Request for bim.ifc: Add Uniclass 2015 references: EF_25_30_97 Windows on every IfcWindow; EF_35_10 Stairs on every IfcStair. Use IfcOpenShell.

First a look at what the model holds.

```python
import ifcopenshell

model = ifcopenshell.open("bim.ifc")
print(model.schema)
print("classifications:", [c.Name for c in model.by_type("IfcClassification")])
for ifc_class in ("IfcDoor", "IfcRoof", "IfcStair", "IfcWall", "IfcWindow"):
    print(ifc_class, len(model.by_type(ifc_class)))
```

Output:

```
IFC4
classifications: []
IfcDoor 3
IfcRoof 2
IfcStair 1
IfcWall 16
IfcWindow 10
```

```python
import ifcopenshell
import ifcopenshell.api.classification

model = ifcopenshell.open("bim.ifc")

system = ifcopenshell.api.classification.add_classification(model, classification="Uniclass 2015")

codes = {
    "IfcWindow": ("EF_25_30_97", "Windows"),
    "IfcStair": ("EF_35_10", "Stairs"),
}
for ifc_class, (code, name) in codes.items():
    products = model.by_type(ifc_class)
    ifcopenshell.api.classification.add_reference(
        model, products=products, classification=system, identification=code, name=name
    )
    print(code, len(products))

model.write("bim-out.ifc")
```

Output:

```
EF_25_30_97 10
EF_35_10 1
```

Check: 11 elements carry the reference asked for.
